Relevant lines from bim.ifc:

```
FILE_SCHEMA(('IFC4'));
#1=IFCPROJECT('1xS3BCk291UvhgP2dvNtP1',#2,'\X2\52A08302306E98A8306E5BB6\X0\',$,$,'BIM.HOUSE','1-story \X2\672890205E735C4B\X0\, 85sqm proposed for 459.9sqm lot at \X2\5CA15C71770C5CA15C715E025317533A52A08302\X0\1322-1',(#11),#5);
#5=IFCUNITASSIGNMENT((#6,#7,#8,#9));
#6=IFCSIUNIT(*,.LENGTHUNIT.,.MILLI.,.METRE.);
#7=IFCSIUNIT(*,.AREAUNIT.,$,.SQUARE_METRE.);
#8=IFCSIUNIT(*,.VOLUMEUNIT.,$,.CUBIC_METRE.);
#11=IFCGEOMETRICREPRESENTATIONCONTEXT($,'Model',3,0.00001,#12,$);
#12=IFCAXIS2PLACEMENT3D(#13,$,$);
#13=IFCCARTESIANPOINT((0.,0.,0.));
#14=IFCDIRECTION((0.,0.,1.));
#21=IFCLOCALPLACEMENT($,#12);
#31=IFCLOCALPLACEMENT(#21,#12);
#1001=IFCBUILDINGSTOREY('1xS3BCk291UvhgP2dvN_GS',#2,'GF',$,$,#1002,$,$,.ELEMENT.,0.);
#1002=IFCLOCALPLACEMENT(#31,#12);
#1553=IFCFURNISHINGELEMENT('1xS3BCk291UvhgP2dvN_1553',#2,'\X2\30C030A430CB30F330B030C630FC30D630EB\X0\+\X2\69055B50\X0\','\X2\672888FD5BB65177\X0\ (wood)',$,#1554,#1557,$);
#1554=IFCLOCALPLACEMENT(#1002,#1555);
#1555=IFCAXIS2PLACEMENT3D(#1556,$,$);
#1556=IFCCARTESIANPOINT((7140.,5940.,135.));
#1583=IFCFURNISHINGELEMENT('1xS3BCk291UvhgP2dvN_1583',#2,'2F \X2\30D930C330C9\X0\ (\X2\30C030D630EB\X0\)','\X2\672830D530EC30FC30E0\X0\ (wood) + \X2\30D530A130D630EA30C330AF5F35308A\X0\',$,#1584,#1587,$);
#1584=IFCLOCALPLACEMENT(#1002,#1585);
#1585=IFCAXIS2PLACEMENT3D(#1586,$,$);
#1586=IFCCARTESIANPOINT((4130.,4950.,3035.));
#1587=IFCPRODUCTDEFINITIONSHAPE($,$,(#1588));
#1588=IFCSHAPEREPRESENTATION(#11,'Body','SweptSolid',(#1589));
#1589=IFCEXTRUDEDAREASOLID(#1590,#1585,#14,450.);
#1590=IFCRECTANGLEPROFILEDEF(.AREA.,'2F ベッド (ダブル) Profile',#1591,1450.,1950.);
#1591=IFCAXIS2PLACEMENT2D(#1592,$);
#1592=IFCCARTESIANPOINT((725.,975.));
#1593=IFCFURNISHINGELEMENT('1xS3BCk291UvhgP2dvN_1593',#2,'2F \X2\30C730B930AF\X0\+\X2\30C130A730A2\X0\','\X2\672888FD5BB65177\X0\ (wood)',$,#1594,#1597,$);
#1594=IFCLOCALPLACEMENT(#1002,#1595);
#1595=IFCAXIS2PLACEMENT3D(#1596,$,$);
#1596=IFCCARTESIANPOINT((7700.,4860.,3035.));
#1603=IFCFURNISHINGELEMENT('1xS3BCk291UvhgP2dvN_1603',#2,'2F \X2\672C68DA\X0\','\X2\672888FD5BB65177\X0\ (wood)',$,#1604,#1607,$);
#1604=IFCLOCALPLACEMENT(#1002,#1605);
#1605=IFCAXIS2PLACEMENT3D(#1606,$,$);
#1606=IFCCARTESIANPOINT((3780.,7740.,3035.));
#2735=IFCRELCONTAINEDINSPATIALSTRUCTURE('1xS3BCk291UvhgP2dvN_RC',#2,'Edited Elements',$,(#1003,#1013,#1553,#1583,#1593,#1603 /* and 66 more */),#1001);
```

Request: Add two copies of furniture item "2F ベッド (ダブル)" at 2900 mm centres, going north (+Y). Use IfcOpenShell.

```python
import numpy as np
import ifcopenshell
import ifcopenshell.api.geometry
import ifcopenshell.api.root
import ifcopenshell.util.element
import ifcopenshell.util.placement

model = ifcopenshell.open("bim.ifc")


def reuse_history(source, copy):
    """copy_class also copies each property set's owner history, people and application; keep the originals."""
    for rel in copy.IsDefinedBy:
        if rel.is_a("IfcRelDefinesByProperties") and (history := rel.RelatingPropertyDefinition.OwnerHistory):
            rel.RelatingPropertyDefinition.OwnerHistory = source.OwnerHistory
            ifcopenshell.util.element.remove_deep2(model, history)


source = model.by_guid("1xS3BCk291UvhgP2dvN_1583")
base = ifcopenshell.util.placement.get_local_placement(source.ObjectPlacement)
step = np.array([0.0, 1.0, 0.0]) * 2900.0

for i in range(1, 3):
    copy = ifcopenshell.api.root.copy_class(model, product=source)
    copy.Representation = ifcopenshell.util.element.copy_deep(
        model, source.Representation, exclude=["IfcGeometricRepresentationContext", "IfcRepresentationMap"]
    )
    reuse_history(source, copy)
    matrix = base.copy()
    matrix[:3, 3] += i * step
    print("added at", matrix[:3, 3].round(3) + 0.0)
    ifcopenshell.api.geometry.edit_object_placement(model, product=copy, matrix=matrix, is_si=False)

model.write("bim_edited.ifc")
```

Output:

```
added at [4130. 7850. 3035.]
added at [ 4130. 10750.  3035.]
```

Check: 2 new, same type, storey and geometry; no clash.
